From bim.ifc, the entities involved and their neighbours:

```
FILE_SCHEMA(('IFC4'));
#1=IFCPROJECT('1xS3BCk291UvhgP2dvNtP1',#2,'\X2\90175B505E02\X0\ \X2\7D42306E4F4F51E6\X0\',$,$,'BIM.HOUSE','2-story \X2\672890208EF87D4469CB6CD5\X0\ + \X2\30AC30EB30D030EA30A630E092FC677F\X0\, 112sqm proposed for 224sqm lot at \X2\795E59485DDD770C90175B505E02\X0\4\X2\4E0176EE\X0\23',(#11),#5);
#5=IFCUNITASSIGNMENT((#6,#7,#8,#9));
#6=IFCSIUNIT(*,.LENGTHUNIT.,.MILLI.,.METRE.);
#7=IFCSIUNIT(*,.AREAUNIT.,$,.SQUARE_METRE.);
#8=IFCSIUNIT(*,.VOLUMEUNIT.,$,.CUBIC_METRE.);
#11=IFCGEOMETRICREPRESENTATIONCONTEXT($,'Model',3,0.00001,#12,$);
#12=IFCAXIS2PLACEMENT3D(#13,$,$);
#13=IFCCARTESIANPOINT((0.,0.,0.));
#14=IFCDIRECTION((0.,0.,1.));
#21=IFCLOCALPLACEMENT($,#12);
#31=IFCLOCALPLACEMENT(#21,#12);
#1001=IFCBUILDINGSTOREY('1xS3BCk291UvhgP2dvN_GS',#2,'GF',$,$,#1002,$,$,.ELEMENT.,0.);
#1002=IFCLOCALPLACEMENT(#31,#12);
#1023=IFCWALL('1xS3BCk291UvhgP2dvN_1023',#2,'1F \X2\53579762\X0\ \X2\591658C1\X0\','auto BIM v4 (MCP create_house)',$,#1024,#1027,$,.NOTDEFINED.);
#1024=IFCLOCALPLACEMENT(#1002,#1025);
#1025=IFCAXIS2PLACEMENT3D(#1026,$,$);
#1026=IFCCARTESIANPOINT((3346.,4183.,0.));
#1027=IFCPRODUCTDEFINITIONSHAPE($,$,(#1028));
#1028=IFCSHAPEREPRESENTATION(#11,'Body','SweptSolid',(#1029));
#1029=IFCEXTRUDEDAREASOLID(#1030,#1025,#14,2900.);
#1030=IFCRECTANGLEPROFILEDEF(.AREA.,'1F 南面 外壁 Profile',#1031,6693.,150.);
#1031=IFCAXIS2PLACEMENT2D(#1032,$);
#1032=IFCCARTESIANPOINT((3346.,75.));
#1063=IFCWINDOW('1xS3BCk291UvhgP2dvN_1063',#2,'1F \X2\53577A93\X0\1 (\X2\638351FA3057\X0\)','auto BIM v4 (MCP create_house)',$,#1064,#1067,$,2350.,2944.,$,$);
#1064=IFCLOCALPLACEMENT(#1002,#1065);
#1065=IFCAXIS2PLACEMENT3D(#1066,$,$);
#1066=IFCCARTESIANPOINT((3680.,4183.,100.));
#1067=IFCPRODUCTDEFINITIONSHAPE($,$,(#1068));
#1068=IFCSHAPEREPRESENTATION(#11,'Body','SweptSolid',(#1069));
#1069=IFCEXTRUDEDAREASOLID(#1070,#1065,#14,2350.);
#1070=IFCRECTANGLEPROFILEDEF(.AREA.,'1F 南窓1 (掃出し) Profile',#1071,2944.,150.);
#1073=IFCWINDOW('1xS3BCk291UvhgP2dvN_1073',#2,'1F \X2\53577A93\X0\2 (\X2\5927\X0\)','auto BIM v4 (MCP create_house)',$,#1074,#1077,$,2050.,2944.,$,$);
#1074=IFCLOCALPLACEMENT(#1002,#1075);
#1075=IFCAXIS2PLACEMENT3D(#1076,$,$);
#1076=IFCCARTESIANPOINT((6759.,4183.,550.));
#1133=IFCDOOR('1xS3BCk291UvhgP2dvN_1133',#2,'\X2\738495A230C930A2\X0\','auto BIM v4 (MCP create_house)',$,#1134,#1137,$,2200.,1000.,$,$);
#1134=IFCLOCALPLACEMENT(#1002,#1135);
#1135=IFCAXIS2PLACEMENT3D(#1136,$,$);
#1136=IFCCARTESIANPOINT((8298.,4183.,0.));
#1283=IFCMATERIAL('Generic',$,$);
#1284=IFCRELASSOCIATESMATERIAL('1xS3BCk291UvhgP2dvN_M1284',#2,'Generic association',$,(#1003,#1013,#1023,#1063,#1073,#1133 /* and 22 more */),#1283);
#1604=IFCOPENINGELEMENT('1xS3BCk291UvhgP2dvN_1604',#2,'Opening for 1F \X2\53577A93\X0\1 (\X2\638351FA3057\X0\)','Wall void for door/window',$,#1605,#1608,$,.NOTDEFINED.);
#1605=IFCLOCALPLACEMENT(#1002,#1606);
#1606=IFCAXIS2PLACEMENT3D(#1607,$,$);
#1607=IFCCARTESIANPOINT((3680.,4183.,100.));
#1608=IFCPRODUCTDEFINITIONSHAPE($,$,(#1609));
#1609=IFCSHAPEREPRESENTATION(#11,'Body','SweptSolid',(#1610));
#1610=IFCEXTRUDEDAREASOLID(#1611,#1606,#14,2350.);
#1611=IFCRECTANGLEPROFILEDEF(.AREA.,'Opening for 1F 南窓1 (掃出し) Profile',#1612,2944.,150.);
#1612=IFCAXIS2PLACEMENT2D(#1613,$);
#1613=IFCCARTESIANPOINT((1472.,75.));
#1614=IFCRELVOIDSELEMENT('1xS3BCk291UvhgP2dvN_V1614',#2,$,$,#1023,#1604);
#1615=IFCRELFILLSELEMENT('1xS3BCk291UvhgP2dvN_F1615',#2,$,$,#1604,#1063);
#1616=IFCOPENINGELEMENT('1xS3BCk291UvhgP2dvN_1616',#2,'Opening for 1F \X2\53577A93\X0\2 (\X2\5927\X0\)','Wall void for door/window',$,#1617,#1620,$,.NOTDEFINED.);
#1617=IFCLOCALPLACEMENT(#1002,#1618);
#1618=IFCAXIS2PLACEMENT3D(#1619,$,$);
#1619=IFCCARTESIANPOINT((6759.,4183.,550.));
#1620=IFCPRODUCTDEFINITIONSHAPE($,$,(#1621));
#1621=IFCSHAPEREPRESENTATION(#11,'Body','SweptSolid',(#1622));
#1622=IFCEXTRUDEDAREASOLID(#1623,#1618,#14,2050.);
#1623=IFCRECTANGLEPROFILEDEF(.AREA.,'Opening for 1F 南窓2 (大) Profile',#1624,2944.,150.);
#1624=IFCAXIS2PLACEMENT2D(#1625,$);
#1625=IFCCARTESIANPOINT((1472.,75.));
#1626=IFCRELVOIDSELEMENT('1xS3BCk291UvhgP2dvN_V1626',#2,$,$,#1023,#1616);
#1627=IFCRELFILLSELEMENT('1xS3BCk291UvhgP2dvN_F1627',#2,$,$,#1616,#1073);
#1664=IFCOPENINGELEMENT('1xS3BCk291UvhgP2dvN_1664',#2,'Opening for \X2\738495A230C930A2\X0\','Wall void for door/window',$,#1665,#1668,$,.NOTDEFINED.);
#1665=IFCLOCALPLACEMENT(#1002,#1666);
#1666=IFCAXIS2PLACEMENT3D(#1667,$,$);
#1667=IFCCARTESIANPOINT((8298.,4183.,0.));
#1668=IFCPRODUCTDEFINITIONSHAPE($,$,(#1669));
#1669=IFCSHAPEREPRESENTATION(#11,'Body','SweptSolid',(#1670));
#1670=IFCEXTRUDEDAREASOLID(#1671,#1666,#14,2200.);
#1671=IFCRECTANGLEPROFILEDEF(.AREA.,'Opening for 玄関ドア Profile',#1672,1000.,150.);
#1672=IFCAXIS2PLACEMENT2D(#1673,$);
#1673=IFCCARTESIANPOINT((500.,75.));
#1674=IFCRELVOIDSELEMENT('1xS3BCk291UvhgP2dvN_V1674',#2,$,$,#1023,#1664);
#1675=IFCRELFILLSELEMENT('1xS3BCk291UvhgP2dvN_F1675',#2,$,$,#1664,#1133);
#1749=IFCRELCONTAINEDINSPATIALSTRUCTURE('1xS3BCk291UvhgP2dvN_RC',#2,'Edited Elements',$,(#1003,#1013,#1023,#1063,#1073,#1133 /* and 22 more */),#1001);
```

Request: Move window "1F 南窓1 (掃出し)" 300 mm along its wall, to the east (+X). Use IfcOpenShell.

```python
import ifcopenshell
import ifcopenshell.api.geometry
import ifcopenshell.util.placement
import ifcopenshell.util.unit

model = ifcopenshell.open("bim.ifc")
unit_scale = ifcopenshell.util.unit.calculate_unit_scale(model)

window = model.by_id(1063)
opening = window.FillsVoids[0].RelatingOpeningElement
wall = opening.VoidsElements[0].RelatingBuildingElement

wall_matrix = ifcopenshell.util.placement.get_local_placement(wall.ObjectPlacement)
shift = wall_matrix[:3, 0] * 0.3 / unit_scale
before = ifcopenshell.util.placement.get_local_placement(window.ObjectPlacement)[:3, 3].copy()

# The window is not placed relative to its opening, so move both.
for product in (opening, window):
    matrix = ifcopenshell.util.placement.get_local_placement(product.ObjectPlacement)
    matrix[:3, 3] += shift
    ifcopenshell.api.geometry.edit_object_placement(model, product=product, matrix=matrix, is_si=False)

after = ifcopenshell.util.placement.get_local_placement(window.ObjectPlacement)[:3, 3]
print("window moved by", (after - before).round(3) + 0.0)

model.write("bim_edited.ifc")
```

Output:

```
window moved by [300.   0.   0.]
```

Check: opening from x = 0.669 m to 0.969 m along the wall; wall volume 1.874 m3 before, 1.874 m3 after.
